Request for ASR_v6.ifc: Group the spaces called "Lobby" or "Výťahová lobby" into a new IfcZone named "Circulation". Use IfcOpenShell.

First a look at what the model holds.

```python
import ifcopenshell

model = ifcopenshell.open("ASR_v6.ifc")
print(model.schema)
seen = {}
for space in model.by_type("IfcSpace"):
    seen[space.LongName] = seen.get(space.LongName, 0) + 1
for name, count in sorted(seen.items(), key=str):
    print(count, "x", name)
print("zones:", [z.Name for z in model.by_type("IfcZone")][:20])
```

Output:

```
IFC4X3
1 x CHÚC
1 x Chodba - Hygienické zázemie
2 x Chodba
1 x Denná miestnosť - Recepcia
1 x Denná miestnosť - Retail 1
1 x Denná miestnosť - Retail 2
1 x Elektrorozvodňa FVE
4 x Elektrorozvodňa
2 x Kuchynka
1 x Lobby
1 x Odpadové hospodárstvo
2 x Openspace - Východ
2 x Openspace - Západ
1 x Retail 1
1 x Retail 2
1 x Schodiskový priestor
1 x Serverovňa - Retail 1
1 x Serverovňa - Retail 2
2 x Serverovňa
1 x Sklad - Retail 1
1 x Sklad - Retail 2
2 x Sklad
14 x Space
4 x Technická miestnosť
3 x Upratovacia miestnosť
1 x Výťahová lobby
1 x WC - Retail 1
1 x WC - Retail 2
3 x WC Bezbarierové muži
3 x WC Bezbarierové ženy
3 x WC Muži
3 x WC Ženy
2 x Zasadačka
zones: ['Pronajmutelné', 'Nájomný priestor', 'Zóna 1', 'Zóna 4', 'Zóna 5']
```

```python
import ifcopenshell
import ifcopenshell.api.group
import ifcopenshell.api.root

model = ifcopenshell.open("ASR_v6.ifc")

names = {"Lobby", "Výťahová lobby"}
spaces = [s for s in model.by_type("IfcSpace") if s.LongName in names]

zone = ifcopenshell.api.root.create_entity(model, ifc_class="IfcZone", name="Circulation")
ifcopenshell.api.group.assign_group(model, products=spaces, group=zone)
print(len(spaces), "spaces in", zone.Name)

model.write("ASR_v6_rev.ifc")
```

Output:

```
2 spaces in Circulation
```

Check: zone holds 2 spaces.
